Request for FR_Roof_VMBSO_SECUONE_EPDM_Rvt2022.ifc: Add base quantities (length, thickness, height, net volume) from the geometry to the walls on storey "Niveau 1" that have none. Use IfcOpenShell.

First a look at what the model holds.

```python
import ifcopenshell
import ifcopenshell.util.element
import ifcopenshell.util.unit

model = ifcopenshell.open("FR_Roof_VMBSO_SECUONE_EPDM_Rvt2022.ifc")
print(model.schema)
for unit_type in ("LENGTHUNIT", "AREAUNIT", "VOLUMEUNIT"):
    print(unit_type, ifcopenshell.util.unit.calculate_unit_scale(model, unit_type))
storey = next(s for s in model.by_type("IfcBuildingStorey") if s.Name == "Niveau 1")
walls = [e for e in ifcopenshell.util.element.get_decomposition(storey) if e.is_a("IfcWall")]
for e in sorted(walls, key=lambda e: e.id()):
    print(e.id(), e.is_a(), e.Name, list(ifcopenshell.util.element.get_psets(e, qtos_only=True)), sep=" | ")
```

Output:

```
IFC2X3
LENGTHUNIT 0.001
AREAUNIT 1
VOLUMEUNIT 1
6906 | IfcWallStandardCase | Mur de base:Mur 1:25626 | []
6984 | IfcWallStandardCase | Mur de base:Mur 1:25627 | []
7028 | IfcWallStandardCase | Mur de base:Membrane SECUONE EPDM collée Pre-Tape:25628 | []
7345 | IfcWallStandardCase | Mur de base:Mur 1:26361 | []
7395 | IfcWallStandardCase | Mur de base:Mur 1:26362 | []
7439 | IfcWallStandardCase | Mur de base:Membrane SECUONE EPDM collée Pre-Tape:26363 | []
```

```python
import ifcopenshell
import ifcopenshell.api.pset
import ifcopenshell.geom
import ifcopenshell.util.element
import ifcopenshell.util.shape
import ifcopenshell.util.unit

model = ifcopenshell.open("FR_Roof_VMBSO_SECUONE_EPDM_Rvt2022.ifc")
unit_scale = ifcopenshell.util.unit.calculate_unit_scale(model)
volume_scale = ifcopenshell.util.unit.calculate_unit_scale(model, "VOLUMEUNIT")
settings = ifcopenshell.geom.settings()

storey = next(s for s in model.by_type("IfcBuildingStorey") if s.Name == "Niveau 1")
walls = [e for e in ifcopenshell.util.element.get_decomposition(storey) if e.is_a("IfcWall")]

for e in sorted(walls, key=lambda e: e.id()):
    if ifcopenshell.util.element.get_psets(e, qtos_only=True, should_inherit=False):
        continue
    # Geometry comes back in metres, in the element's own axes.
    shape = ifcopenshell.geom.create_shape(settings, e)
    values = {
        "Length": ifcopenshell.util.shape.get_x(shape.geometry) / unit_scale,
        "Width": ifcopenshell.util.shape.get_y(shape.geometry) / unit_scale,
        "Height": ifcopenshell.util.shape.get_z(shape.geometry) / unit_scale,
        "NetVolume": ifcopenshell.util.shape.get_volume(shape.geometry) / volume_scale,
    }
    qto = ifcopenshell.api.pset.add_qto(model, product=e, name="BaseQuantities")
    ifcopenshell.api.pset.edit_qto(model, qto=qto, properties=values)
    print(e.id(), {k: round(v, 3) for k, v in values.items()})

model.write("FR_Roof_VMBSO_SECUONE_EPDM_Rvt2022-out.ifc")
```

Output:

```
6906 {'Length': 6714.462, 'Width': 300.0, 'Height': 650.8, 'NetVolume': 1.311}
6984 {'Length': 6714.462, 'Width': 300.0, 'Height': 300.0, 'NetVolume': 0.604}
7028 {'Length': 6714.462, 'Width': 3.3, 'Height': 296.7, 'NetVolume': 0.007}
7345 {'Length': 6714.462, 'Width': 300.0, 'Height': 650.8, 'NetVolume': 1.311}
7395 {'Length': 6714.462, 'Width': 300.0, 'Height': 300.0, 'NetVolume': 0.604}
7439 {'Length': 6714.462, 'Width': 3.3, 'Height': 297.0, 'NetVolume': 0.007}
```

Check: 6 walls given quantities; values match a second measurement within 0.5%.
